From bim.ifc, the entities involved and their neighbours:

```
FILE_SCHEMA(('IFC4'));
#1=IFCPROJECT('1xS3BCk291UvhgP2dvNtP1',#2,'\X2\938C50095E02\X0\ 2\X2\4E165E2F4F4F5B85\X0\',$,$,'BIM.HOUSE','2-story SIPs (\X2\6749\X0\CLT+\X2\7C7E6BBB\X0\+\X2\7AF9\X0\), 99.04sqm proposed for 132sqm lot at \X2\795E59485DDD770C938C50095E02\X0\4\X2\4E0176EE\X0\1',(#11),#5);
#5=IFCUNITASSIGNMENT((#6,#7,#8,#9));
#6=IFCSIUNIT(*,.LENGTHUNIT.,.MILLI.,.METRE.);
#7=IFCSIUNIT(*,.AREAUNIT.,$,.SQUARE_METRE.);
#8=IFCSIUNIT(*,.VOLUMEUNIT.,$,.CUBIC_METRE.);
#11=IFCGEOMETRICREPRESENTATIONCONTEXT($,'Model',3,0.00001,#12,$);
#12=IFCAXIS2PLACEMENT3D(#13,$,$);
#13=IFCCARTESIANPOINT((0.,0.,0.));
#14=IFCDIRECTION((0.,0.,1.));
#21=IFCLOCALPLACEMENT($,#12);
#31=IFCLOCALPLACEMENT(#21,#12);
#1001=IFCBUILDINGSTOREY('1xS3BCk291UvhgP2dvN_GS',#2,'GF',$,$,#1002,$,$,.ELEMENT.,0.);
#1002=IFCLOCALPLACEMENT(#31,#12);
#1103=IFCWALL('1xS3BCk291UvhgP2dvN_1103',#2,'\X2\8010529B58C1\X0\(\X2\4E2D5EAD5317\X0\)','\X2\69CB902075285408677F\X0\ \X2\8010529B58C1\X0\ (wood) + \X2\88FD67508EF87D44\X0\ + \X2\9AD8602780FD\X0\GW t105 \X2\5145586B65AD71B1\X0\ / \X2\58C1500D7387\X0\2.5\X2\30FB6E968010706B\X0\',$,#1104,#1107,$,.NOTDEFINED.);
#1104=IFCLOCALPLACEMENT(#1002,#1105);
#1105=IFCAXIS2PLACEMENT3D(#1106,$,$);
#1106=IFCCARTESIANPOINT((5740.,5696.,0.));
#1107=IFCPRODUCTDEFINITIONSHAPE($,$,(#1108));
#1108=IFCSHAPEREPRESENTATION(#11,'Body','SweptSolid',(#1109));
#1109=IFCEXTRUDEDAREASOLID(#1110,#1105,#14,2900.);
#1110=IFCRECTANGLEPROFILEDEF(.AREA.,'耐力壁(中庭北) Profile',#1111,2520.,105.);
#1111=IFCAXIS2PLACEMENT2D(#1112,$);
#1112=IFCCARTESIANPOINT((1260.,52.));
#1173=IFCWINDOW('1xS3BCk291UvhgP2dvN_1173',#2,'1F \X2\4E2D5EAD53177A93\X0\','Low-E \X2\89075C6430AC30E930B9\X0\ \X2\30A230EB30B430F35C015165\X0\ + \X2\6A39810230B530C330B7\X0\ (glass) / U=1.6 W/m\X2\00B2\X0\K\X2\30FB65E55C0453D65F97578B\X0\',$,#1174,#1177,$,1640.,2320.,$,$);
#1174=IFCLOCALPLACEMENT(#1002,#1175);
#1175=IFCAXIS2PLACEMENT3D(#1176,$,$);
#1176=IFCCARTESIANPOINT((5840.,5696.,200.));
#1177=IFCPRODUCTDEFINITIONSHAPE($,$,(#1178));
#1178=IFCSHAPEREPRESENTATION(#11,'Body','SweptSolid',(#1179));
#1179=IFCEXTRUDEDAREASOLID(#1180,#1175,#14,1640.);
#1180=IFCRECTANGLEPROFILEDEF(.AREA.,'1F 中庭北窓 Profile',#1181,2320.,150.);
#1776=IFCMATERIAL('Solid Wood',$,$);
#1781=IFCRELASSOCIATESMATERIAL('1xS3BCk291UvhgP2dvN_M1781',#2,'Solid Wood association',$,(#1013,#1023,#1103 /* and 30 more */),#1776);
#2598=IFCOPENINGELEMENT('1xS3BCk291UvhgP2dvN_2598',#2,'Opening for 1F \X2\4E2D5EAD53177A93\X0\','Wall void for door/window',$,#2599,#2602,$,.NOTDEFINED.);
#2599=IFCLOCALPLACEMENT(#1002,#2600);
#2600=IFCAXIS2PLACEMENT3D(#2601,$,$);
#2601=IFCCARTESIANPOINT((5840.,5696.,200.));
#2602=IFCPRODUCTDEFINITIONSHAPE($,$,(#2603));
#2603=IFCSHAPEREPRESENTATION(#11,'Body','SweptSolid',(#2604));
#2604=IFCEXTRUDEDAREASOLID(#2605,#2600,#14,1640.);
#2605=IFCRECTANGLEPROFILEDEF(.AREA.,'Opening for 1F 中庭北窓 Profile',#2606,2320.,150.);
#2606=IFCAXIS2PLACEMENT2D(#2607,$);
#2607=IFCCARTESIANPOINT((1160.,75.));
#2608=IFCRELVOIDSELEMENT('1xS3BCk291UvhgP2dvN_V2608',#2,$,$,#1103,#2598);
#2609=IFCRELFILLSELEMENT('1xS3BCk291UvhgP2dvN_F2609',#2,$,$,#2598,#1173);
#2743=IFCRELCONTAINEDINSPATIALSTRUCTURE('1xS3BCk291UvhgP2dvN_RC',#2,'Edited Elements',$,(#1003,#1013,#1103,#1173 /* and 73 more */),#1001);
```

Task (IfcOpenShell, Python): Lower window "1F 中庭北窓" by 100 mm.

```python
import numpy as np
import ifcopenshell
import ifcopenshell.api.geometry
import ifcopenshell.util.placement
import ifcopenshell.util.unit

model = ifcopenshell.open("bim.ifc")
unit_scale = ifcopenshell.util.unit.calculate_unit_scale(model)

window = model.by_guid("1xS3BCk291UvhgP2dvN_1173")
opening = window.FillsVoids[0].RelatingOpeningElement
dz = -0.1 / unit_scale

shift = np.array([0.0, 0.0, dz])
# The window is not placed relative to its opening, so move both.
for product in (opening, window):
    matrix = ifcopenshell.util.placement.get_local_placement(product.ObjectPlacement)
    matrix[:3, 3] += shift
    ifcopenshell.api.geometry.edit_object_placement(model, product=product, matrix=matrix, is_si=False)

print(f"moved by {dz * unit_scale:+.3f} m")

model.write("bim_updated.ifc")
```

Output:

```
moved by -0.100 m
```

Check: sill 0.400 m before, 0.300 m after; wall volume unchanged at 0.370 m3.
